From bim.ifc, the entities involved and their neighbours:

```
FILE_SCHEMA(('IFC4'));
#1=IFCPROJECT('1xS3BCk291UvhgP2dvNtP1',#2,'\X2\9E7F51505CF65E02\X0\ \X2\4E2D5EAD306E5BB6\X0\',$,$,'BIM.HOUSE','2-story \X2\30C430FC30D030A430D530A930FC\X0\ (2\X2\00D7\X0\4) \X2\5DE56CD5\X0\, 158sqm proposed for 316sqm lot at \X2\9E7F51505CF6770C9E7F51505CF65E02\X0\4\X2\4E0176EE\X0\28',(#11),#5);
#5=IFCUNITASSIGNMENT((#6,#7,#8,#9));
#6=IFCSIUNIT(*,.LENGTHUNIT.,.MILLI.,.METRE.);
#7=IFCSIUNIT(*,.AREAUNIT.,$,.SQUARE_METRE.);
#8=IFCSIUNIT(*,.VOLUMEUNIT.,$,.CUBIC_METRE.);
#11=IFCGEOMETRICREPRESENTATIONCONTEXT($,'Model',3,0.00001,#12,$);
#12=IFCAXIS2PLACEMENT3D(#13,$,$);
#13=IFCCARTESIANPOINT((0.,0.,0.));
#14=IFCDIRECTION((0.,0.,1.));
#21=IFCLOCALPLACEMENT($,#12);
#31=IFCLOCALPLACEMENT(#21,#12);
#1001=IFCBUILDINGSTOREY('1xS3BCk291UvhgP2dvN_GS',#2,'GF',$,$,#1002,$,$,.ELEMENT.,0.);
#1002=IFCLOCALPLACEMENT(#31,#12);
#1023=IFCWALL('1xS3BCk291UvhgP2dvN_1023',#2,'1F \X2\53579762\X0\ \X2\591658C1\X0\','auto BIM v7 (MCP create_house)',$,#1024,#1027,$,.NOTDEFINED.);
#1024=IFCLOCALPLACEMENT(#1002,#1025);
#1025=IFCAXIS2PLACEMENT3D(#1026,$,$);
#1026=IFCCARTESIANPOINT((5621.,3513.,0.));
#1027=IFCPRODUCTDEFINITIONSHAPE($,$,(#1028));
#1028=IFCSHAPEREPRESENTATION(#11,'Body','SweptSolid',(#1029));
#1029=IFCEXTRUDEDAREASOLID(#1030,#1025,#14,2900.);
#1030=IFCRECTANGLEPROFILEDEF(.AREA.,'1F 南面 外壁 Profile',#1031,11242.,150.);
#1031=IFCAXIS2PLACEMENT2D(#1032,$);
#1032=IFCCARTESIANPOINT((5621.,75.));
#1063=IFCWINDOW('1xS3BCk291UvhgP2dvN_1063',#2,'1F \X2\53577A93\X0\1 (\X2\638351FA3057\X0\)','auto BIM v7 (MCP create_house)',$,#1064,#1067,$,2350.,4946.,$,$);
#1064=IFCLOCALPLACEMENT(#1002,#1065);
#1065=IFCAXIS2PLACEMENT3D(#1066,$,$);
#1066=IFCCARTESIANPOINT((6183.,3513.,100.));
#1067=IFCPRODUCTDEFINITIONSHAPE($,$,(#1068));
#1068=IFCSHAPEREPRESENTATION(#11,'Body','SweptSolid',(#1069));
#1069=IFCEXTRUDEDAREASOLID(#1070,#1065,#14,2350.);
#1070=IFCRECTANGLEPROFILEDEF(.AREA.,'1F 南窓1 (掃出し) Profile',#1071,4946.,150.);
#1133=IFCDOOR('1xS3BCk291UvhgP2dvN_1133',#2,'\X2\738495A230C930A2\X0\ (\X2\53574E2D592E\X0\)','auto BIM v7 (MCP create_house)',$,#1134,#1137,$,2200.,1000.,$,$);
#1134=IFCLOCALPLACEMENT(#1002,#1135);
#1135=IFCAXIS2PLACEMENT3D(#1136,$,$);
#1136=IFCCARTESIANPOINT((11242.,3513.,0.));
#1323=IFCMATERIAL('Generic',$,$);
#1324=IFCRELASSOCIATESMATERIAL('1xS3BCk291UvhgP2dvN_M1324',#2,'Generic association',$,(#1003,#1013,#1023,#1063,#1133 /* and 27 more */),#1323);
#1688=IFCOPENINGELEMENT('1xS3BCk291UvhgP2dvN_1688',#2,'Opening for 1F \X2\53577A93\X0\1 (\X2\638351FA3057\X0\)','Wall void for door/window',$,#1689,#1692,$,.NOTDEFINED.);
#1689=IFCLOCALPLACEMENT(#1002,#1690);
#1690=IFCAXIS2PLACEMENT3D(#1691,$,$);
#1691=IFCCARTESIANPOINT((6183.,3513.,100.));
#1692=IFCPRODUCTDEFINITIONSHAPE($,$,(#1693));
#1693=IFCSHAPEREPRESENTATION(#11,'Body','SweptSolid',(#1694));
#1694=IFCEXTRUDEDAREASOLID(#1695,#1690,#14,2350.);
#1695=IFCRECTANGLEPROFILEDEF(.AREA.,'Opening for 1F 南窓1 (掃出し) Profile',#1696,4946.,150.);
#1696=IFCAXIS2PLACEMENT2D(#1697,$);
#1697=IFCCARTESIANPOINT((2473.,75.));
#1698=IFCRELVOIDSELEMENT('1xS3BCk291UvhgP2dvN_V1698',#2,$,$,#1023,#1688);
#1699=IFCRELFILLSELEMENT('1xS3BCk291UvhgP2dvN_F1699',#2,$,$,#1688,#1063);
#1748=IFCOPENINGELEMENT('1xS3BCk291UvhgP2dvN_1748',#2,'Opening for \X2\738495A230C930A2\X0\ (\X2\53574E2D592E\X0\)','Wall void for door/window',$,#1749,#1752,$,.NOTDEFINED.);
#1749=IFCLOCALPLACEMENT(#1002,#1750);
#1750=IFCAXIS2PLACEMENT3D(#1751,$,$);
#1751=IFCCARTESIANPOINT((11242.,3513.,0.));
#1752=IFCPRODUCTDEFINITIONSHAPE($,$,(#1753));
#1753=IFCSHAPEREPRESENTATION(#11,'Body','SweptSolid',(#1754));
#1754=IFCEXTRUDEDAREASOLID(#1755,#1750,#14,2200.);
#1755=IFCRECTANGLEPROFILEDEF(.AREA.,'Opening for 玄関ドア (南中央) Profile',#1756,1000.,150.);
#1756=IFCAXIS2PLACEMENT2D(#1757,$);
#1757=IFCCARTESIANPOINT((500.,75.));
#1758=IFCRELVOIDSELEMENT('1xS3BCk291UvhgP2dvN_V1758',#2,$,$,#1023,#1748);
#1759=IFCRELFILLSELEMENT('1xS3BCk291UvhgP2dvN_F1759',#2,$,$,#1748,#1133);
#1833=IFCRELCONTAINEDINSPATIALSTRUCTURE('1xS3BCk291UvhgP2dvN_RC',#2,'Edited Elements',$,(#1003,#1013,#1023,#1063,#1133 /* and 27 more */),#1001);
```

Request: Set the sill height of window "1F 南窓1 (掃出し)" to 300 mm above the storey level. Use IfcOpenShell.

```python
import numpy as np
import ifcopenshell
import ifcopenshell.api.geometry
import ifcopenshell.geom
import ifcopenshell.util.element
import ifcopenshell.util.placement
import ifcopenshell.util.shape
import ifcopenshell.util.unit

model = ifcopenshell.open("bim.ifc")
unit_scale = ifcopenshell.util.unit.calculate_unit_scale(model)

window = model.by_guid("1xS3BCk291UvhgP2dvN_1063")
opening = window.FillsVoids[0].RelatingOpeningElement
storey = ifcopenshell.util.element.get_container(window, ifc_class="IfcBuildingStorey")
level = ifcopenshell.util.placement.get_local_placement(storey.ObjectPlacement)[2, 3]

# The opening's origin need not be at the sill, so measure its lowest point.
shape = ifcopenshell.geom.create_shape(ifcopenshell.geom.settings(), opening)
bottom = ifcopenshell.util.shape.get_shape_bottom_elevation(shape, shape.geometry) / unit_scale
dz = level + 0.3 / unit_scale - bottom

shift = np.array([0.0, 0.0, dz])
# The window is not placed relative to its opening, so move both.
for product in (opening, window):
    matrix = ifcopenshell.util.placement.get_local_placement(product.ObjectPlacement)
    matrix[:3, 3] += shift
    ifcopenshell.api.geometry.edit_object_placement(model, product=product, matrix=matrix, is_si=False)

print(f"moved by {dz * unit_scale:+.3f} m")

model.write("bim-out.ifc")
```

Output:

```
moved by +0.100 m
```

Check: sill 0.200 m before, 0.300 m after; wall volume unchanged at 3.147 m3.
